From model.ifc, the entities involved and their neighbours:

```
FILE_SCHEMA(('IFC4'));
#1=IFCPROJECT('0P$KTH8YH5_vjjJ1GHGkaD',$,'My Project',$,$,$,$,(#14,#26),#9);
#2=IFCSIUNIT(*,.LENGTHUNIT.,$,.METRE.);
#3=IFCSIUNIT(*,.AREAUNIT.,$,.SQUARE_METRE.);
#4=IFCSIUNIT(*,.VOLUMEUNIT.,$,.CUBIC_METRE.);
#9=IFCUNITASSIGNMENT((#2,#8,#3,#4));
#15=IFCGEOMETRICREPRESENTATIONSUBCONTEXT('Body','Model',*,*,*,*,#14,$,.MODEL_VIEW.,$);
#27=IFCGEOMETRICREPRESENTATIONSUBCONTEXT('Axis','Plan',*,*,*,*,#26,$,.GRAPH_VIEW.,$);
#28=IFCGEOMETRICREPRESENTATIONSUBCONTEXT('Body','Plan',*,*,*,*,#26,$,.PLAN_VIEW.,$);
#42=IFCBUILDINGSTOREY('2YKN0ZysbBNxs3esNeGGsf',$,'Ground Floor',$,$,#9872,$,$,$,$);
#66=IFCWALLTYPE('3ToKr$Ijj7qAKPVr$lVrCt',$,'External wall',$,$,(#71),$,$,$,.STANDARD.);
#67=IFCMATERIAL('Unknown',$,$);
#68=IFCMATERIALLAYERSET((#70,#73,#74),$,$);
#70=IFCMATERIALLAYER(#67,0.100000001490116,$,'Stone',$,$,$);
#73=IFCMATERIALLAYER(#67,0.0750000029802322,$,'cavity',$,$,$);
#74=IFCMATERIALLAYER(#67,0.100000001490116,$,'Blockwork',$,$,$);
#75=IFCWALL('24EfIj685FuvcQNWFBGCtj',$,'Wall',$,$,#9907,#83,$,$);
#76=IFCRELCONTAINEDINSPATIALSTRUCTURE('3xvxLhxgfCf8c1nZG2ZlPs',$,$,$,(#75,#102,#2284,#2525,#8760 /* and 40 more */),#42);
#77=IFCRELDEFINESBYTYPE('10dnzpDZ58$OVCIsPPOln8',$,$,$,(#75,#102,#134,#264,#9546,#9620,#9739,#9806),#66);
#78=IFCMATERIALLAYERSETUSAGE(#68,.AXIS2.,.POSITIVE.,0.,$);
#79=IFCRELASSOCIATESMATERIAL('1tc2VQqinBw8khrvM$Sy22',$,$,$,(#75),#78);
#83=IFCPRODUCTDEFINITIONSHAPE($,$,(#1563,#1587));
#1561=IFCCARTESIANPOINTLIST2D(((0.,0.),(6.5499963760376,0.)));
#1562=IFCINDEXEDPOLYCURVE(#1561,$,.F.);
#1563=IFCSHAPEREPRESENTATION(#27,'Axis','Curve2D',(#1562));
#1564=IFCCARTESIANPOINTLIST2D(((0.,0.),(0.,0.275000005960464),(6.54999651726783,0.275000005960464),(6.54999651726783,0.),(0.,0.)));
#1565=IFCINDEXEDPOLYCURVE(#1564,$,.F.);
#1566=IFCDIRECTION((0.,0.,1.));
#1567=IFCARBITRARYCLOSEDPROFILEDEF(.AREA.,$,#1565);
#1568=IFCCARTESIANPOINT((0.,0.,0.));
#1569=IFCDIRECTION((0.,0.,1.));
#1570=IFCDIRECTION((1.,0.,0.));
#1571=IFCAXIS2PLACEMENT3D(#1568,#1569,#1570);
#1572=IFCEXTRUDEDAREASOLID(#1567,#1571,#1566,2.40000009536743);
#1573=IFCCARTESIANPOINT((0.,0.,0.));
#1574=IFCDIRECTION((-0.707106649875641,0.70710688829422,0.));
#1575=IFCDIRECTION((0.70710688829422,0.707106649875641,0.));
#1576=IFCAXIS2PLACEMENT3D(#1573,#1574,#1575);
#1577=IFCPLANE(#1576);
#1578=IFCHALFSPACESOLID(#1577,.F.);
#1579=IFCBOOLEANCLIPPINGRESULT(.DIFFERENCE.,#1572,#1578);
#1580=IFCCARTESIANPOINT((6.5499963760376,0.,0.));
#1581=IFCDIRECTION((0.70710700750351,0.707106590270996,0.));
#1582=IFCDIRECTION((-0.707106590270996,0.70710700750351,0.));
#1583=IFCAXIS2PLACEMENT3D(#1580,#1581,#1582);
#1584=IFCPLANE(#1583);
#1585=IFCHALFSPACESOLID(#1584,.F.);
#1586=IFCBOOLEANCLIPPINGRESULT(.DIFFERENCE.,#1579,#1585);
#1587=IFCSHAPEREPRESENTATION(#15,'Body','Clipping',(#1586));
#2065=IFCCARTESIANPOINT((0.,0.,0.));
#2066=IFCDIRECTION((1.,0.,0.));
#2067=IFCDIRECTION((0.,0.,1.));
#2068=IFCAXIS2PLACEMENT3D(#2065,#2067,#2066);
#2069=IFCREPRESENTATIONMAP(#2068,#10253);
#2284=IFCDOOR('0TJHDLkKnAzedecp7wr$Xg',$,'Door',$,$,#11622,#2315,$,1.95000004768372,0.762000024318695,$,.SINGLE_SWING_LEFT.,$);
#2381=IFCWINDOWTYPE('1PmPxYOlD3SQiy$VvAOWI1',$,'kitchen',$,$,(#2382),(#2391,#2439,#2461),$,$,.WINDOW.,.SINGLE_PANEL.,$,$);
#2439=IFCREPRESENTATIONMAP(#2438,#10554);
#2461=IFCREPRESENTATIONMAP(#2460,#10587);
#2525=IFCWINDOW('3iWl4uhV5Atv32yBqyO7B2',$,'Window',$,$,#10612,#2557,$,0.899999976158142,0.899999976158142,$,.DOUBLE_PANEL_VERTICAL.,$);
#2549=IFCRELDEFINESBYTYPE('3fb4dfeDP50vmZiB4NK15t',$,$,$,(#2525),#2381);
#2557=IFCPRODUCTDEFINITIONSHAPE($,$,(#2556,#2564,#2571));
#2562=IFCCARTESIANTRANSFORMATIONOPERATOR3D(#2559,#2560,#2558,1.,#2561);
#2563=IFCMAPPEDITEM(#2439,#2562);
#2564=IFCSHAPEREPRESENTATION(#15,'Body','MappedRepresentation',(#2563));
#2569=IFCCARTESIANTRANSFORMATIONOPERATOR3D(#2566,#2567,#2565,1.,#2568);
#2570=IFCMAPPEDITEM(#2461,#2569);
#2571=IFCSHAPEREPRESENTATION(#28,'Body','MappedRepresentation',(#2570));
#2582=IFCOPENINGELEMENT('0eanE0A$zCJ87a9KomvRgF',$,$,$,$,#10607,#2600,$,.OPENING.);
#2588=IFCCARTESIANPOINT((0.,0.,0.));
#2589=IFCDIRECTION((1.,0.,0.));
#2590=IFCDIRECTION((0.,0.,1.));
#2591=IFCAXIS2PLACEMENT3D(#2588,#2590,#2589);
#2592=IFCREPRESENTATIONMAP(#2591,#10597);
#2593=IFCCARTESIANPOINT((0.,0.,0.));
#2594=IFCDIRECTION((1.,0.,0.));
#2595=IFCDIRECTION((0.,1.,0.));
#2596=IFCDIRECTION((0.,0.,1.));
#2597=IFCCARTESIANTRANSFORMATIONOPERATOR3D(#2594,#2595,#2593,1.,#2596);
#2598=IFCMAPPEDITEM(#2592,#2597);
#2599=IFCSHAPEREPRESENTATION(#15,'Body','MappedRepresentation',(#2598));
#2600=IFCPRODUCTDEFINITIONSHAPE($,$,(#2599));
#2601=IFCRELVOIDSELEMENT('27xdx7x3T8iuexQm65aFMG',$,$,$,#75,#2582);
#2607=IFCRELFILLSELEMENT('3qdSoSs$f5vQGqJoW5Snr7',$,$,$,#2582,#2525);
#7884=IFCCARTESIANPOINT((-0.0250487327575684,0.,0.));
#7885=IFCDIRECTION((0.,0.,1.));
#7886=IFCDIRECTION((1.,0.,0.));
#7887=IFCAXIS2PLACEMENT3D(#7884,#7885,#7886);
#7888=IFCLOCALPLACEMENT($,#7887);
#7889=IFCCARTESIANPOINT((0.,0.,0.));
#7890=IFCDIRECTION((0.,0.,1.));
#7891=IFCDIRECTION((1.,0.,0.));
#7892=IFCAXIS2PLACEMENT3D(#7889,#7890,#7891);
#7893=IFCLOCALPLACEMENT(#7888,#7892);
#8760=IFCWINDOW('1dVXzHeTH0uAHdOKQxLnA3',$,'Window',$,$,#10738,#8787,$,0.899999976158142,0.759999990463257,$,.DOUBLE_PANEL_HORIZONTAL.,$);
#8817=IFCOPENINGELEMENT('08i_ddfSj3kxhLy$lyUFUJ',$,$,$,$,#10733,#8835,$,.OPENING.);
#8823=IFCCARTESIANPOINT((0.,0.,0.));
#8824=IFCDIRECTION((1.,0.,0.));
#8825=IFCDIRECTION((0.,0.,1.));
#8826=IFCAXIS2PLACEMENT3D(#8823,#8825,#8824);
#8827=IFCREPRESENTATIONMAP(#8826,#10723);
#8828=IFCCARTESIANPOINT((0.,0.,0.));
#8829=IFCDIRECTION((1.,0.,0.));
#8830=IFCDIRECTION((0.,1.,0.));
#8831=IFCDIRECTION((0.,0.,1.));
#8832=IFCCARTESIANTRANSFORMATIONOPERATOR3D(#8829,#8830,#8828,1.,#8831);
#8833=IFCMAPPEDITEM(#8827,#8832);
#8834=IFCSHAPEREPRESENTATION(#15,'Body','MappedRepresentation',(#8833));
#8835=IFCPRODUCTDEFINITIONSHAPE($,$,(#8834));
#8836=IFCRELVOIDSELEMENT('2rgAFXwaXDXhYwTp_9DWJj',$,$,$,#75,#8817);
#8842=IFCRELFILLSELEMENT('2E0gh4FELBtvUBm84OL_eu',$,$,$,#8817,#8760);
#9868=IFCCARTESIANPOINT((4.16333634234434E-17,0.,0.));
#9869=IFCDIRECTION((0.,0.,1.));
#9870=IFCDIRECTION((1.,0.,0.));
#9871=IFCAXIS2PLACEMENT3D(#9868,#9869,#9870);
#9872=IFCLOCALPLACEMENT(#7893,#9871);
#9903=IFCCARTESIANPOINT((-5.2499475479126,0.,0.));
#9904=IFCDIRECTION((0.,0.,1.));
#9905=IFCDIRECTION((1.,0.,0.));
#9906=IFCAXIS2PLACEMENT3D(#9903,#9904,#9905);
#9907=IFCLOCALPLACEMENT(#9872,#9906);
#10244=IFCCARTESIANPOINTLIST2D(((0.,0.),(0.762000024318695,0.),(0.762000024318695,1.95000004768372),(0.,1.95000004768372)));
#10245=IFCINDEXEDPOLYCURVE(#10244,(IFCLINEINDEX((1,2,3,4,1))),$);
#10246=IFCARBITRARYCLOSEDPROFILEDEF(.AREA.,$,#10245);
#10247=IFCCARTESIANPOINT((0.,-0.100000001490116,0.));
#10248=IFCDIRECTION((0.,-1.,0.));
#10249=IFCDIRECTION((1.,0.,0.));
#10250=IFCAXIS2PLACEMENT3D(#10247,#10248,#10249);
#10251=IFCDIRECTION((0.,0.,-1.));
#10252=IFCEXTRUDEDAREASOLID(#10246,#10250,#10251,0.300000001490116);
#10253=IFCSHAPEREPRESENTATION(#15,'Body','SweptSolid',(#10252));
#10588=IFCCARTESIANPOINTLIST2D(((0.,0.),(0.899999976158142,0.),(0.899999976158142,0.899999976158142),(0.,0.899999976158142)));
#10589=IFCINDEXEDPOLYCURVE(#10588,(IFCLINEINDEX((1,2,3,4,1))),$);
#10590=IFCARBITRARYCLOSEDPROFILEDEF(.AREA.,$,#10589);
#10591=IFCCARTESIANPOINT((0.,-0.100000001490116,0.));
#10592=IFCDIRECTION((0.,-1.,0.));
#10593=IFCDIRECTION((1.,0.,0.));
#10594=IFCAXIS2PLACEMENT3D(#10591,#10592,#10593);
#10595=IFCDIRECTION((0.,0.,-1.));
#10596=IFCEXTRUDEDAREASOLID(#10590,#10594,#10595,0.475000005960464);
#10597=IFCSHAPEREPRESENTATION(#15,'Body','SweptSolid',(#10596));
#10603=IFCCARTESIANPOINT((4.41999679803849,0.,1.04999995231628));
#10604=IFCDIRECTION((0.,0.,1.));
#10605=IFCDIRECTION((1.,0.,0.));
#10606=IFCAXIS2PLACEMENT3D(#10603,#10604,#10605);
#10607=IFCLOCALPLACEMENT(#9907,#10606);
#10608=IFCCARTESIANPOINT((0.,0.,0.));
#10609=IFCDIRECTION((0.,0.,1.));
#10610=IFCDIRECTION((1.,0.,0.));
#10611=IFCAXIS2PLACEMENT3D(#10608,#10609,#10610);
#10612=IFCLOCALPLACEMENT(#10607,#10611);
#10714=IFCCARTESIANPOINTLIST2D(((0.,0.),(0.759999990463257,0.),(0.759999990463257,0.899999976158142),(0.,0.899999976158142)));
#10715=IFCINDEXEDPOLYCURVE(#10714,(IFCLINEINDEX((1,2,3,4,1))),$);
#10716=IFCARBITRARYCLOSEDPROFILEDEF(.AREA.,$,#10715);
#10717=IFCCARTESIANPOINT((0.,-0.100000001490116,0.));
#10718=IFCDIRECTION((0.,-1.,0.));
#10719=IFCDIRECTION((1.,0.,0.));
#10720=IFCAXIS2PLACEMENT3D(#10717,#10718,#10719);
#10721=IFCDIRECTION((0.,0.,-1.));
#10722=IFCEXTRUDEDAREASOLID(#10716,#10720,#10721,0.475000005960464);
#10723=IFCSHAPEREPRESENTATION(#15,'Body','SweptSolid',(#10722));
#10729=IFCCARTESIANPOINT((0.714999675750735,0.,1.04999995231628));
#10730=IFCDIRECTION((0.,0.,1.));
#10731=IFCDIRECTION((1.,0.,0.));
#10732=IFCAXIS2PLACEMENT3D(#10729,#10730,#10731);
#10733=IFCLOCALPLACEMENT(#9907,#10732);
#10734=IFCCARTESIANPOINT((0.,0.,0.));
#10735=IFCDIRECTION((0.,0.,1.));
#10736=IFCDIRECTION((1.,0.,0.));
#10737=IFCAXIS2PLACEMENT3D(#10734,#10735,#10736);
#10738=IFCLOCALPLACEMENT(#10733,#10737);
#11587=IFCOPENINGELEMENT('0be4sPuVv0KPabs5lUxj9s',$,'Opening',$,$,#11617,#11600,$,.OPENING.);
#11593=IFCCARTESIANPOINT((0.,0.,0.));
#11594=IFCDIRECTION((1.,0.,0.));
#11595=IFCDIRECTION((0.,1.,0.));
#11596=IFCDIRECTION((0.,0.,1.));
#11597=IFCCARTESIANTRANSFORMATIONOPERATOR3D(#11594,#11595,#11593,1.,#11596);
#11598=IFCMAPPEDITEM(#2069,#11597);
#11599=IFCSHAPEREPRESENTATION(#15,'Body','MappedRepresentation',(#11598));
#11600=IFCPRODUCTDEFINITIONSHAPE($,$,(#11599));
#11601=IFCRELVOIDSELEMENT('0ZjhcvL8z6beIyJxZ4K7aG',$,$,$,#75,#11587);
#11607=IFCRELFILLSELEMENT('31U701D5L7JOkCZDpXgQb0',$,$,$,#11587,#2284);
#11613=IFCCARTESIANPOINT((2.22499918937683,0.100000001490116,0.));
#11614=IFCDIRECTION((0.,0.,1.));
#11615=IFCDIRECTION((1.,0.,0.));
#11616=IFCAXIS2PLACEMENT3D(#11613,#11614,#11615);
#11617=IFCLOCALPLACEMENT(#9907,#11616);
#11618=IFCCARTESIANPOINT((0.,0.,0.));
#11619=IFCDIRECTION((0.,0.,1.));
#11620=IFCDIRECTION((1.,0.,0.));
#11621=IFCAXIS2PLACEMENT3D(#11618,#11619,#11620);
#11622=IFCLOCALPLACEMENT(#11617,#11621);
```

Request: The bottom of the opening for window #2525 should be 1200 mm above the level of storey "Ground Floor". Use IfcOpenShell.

```python
import numpy as np
import ifcopenshell
import ifcopenshell.api.geometry
import ifcopenshell.geom
import ifcopenshell.util.element
import ifcopenshell.util.placement
import ifcopenshell.util.shape
import ifcopenshell.util.unit

model = ifcopenshell.open("model.ifc")
unit_scale = ifcopenshell.util.unit.calculate_unit_scale(model)

window = model.by_guid("3iWl4uhV5Atv32yBqyO7B2")
opening = window.FillsVoids[0].RelatingOpeningElement
storey = ifcopenshell.util.element.get_container(window, ifc_class="IfcBuildingStorey")
level = ifcopenshell.util.placement.get_local_placement(storey.ObjectPlacement)[2, 3]

# The opening's origin need not be at the sill, so measure its lowest point.
shape = ifcopenshell.geom.create_shape(ifcopenshell.geom.settings(), opening)
bottom = ifcopenshell.util.shape.get_shape_bottom_elevation(shape, shape.geometry) / unit_scale
dz = level + 1.2 / unit_scale - bottom

shift = np.array([0.0, 0.0, dz])
# The window is placed relative to its opening, so it follows when the opening moves.
matrix = ifcopenshell.util.placement.get_local_placement(opening.ObjectPlacement)
matrix[:3, 3] += shift
ifcopenshell.api.geometry.edit_object_placement(
    model, product=opening, matrix=matrix, is_si=False, should_transform_children=True
)

print(f"moved by {dz * unit_scale:+.3f} m")

model.write("model_v2.ifc")
```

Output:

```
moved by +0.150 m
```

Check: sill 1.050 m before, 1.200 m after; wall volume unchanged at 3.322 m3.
